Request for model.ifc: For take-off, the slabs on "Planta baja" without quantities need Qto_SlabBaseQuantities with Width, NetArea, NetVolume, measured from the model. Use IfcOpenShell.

First a look at what the model holds.

```python
import ifcopenshell
import ifcopenshell.util.element
import ifcopenshell.util.unit

model = ifcopenshell.open("model.ifc")
print(model.schema)
for unit_type in ("LENGTHUNIT", "AREAUNIT", "VOLUMEUNIT"):
    print(unit_type, ifcopenshell.util.unit.calculate_unit_scale(model, unit_type))
storey = next(s for s in model.by_type("IfcBuildingStorey") if s.Name == "Planta baja")
slabs = [e for e in ifcopenshell.util.element.get_decomposition(storey) if e.is_a("IfcSlab")]
for e in sorted(slabs, key=lambda e: e.id()):
    print(e.id(), e.is_a(), e.Name, list(ifcopenshell.util.element.get_psets(e, qtos_only=True)), sep=" | ")
```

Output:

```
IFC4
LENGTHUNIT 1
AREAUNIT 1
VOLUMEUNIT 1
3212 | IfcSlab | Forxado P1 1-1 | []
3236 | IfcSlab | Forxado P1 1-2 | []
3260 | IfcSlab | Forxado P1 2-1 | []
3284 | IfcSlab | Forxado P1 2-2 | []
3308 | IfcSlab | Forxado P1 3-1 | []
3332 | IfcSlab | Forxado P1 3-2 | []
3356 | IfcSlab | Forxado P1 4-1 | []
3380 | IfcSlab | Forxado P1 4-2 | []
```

```python
import ifcopenshell
import ifcopenshell.api.pset
import ifcopenshell.geom
import ifcopenshell.util.element
import ifcopenshell.util.shape
import ifcopenshell.util.unit

model = ifcopenshell.open("model.ifc")
unit_scale = ifcopenshell.util.unit.calculate_unit_scale(model)
area_scale = ifcopenshell.util.unit.calculate_unit_scale(model, "AREAUNIT")
volume_scale = ifcopenshell.util.unit.calculate_unit_scale(model, "VOLUMEUNIT")
settings = ifcopenshell.geom.settings()

storey = next(s for s in model.by_type("IfcBuildingStorey") if s.Name == "Planta baja")
slabs = [e for e in ifcopenshell.util.element.get_decomposition(storey) if e.is_a("IfcSlab")]

for e in sorted(slabs, key=lambda e: e.id()):
    if ifcopenshell.util.element.get_psets(e, qtos_only=True, should_inherit=False):
        continue
    # Geometry comes back in metres, in the element's own axes.
    shape = ifcopenshell.geom.create_shape(settings, e)
    values = {
        "Width": ifcopenshell.util.shape.get_z(shape.geometry) / unit_scale,
        "NetArea": ifcopenshell.util.shape.get_footprint_area(shape.geometry) / area_scale,
        "NetVolume": ifcopenshell.util.shape.get_volume(shape.geometry) / volume_scale,
    }
    qto = ifcopenshell.api.pset.add_qto(model, product=e, name="Qto_SlabBaseQuantities")
    ifcopenshell.api.pset.edit_qto(model, qto=qto, properties=values)
    print(e.id(), {k: round(v, 3) for k, v in values.items()})

model.write("model_v2.ifc")
```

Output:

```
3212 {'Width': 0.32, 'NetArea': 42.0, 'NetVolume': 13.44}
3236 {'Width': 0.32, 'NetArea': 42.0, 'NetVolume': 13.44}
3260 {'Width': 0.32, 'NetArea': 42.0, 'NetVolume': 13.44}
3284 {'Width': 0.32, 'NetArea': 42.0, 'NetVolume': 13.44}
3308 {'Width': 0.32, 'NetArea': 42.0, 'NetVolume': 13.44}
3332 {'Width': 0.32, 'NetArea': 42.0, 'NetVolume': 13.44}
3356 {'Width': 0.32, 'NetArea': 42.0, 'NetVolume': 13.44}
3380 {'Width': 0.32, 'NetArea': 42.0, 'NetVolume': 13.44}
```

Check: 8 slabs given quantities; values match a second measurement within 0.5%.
